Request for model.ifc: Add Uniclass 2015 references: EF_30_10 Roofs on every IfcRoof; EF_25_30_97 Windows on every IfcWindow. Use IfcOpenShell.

First a look at what the model holds.

```python
import ifcopenshell

model = ifcopenshell.open("model.ifc")
print(model.schema)
print("classifications:", [c.Name for c in model.by_type("IfcClassification")])
for ifc_class in ("IfcDoor", "IfcRoof", "IfcStair", "IfcWall", "IfcWindow"):
    print(ifc_class, len(model.by_type(ifc_class)))
```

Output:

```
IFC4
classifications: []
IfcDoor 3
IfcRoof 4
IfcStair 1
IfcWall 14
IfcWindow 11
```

```python
import ifcopenshell
import ifcopenshell.api.classification

model = ifcopenshell.open("model.ifc")

system = ifcopenshell.api.classification.add_classification(model, classification="Uniclass 2015")

codes = {
    "IfcRoof": ("EF_30_10", "Roofs"),
    "IfcWindow": ("EF_25_30_97", "Windows"),
}
for ifc_class, (code, name) in codes.items():
    products = model.by_type(ifc_class)
    ifcopenshell.api.classification.add_reference(
        model, products=products, classification=system, identification=code, name=name
    )
    print(code, len(products))

model.write("model-out.ifc")
```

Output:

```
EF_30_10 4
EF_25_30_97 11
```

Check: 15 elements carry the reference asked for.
